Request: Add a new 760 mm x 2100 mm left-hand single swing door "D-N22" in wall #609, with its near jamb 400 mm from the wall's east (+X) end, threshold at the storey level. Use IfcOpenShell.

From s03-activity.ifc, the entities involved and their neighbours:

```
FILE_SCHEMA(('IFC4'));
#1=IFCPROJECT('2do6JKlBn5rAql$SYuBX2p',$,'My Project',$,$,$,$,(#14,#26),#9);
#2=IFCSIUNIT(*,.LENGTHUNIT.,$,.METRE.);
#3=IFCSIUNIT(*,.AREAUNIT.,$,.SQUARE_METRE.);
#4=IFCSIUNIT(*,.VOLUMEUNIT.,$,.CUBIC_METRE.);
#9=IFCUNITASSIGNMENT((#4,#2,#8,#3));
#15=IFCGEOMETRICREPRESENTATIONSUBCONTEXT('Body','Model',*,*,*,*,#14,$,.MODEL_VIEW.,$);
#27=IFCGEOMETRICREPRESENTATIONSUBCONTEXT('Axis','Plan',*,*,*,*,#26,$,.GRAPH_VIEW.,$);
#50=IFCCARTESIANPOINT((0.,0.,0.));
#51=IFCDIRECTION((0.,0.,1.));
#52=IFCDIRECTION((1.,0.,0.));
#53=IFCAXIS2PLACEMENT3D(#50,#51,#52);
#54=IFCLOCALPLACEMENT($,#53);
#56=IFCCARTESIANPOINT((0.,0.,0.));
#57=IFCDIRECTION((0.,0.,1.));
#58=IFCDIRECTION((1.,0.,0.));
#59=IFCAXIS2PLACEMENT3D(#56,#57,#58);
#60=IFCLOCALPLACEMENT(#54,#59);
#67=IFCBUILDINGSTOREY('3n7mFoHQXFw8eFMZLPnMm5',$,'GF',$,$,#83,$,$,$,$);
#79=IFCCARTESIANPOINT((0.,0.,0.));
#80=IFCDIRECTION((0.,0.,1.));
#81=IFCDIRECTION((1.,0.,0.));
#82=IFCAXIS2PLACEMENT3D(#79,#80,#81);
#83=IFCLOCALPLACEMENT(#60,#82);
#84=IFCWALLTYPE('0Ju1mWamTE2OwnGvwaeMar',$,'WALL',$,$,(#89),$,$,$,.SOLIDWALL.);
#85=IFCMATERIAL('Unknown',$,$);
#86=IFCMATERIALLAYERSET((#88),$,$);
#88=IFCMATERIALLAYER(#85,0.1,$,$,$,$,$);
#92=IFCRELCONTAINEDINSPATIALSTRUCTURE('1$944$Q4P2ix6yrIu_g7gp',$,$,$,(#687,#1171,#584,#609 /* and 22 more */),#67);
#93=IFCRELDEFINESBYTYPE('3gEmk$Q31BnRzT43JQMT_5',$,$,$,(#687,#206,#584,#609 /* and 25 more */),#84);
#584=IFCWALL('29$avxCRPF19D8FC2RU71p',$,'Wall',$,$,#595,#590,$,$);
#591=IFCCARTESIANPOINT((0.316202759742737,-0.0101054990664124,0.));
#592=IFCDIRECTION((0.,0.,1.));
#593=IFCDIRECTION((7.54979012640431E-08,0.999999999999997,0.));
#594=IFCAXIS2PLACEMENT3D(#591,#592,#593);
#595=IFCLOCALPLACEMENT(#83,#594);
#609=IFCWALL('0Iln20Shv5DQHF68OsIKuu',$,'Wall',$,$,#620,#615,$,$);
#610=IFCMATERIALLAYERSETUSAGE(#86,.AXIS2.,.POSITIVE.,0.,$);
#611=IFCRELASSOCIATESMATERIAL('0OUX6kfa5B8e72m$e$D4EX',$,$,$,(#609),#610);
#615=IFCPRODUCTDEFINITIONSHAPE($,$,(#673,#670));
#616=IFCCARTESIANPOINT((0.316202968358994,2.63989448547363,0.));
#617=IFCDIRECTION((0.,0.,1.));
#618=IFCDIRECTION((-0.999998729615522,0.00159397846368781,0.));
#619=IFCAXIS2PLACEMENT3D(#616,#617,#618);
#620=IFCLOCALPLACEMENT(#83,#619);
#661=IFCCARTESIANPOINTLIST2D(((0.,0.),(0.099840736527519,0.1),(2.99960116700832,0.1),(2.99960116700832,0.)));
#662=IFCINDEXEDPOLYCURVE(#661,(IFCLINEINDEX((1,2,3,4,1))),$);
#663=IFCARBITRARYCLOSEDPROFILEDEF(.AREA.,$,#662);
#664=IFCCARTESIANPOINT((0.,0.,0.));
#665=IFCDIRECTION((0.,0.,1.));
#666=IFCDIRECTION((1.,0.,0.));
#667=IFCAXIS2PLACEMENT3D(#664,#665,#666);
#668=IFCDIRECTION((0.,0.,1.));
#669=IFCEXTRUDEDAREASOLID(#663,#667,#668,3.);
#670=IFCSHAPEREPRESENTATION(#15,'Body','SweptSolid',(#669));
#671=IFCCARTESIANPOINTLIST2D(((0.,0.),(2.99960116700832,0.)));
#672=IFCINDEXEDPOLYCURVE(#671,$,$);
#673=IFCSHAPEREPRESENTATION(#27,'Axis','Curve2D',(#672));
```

```python
import numpy as np
import ifcopenshell
import ifcopenshell.api.feature
import ifcopenshell.api.geometry
import ifcopenshell.api.root
import ifcopenshell.api.spatial
import ifcopenshell.geom
import ifcopenshell.util.element
import ifcopenshell.util.placement
import ifcopenshell.util.representation
import ifcopenshell.util.shape
import ifcopenshell.util.unit

model = ifcopenshell.open("s03-activity.ifc")
unit_scale = ifcopenshell.util.unit.calculate_unit_scale(model)
settings = ifcopenshell.geom.settings()


def volume(element):
    """Net volume in cubic metres, openings subtracted."""
    shape = ifcopenshell.geom.create_shape(settings, element)
    return ifcopenshell.util.shape.get_volume(shape.geometry)


wall = model.by_guid("0Iln20Shv5DQHF68OsIKuu")
storey = ifcopenshell.util.element.get_container(wall, ifc_class="IfcBuildingStorey")
context = ifcopenshell.util.representation.get_context(model, "Model", "Body", "MODEL_VIEW")
before = volume(wall)

width, height, from_end, sill = 0.76, 2.1, 0.4, 0.0  # metres

# The wall runs along its own X axis, and the end named is its -X end.
wall_shape = ifcopenshell.geom.create_shape(settings, wall)
x, y, z = ifcopenshell.util.shape.get_vertices(wall_shape.geometry).T
start = x.min() + from_end
face, thickness = float(y.min()), float(y.max() - y.min())
wall_matrix = ifcopenshell.util.placement.get_local_placement(wall.ObjectPlacement)
level = ifcopenshell.util.placement.get_local_placement(storey.ObjectPlacement)[2, 3]


def in_wall(x, y):
    """Placement at x, y metres in the wall's axes, at sill height."""
    matrix = wall_matrix.copy()
    matrix[:, 3] = wall_matrix @ np.array([x / unit_scale, y / unit_scale, 0.0, 1.0])
    matrix[2, 3] = level + sill / unit_scale
    return matrix


# Opening: a box that overshoots both wall faces by 50 mm.
opening = ifcopenshell.api.root.create_entity(model, ifc_class="IfcOpeningElement", predefined_type="OPENING")
box = ifcopenshell.api.geometry.add_wall_representation(
    model, context=context, length=width, height=height, thickness=thickness + 0.1
)
ifcopenshell.api.geometry.assign_representation(model, product=opening, representation=box)
ifcopenshell.api.geometry.edit_object_placement(model, product=opening, matrix=in_wall(start, face - 0.05), is_si=False)
ifcopenshell.api.feature.add_feature(model, feature=opening, element=wall)

door = ifcopenshell.api.root.create_entity(model, ifc_class="IfcDoor", name="D-N22", predefined_type="DOOR")
door.OverallWidth, door.OverallHeight = width / unit_scale, height / unit_scale
door.OperationType = "SINGLE_SWING_LEFT"
body = ifcopenshell.api.geometry.add_door_representation(
    model,
    context=context,
    overall_width=door.OverallWidth,
    overall_height=door.OverallHeight,
    operation_type="SINGLE_SWING_LEFT",
    lining_properties={"LiningDepth": thickness / unit_scale, "ThresholdDepth": thickness / unit_scale},
)
ifcopenshell.api.geometry.assign_representation(model, product=door, representation=body)
ifcopenshell.api.spatial.assign_container(model, products=[door], relating_structure=storey)
ifcopenshell.api.feature.add_filling(model, opening=opening, element=door)

# The lining spans the wall, so the door starts at the wall face.
ifcopenshell.api.geometry.edit_object_placement(model, product=door, matrix=in_wall(start, face), is_si=False)

after = volume(wall)

print(f"wall volume {before:.3f} -> {after:.3f} m3")

model.write("s03-activity-out.ifc")
```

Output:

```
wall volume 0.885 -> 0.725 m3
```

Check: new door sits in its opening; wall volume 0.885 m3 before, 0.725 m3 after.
